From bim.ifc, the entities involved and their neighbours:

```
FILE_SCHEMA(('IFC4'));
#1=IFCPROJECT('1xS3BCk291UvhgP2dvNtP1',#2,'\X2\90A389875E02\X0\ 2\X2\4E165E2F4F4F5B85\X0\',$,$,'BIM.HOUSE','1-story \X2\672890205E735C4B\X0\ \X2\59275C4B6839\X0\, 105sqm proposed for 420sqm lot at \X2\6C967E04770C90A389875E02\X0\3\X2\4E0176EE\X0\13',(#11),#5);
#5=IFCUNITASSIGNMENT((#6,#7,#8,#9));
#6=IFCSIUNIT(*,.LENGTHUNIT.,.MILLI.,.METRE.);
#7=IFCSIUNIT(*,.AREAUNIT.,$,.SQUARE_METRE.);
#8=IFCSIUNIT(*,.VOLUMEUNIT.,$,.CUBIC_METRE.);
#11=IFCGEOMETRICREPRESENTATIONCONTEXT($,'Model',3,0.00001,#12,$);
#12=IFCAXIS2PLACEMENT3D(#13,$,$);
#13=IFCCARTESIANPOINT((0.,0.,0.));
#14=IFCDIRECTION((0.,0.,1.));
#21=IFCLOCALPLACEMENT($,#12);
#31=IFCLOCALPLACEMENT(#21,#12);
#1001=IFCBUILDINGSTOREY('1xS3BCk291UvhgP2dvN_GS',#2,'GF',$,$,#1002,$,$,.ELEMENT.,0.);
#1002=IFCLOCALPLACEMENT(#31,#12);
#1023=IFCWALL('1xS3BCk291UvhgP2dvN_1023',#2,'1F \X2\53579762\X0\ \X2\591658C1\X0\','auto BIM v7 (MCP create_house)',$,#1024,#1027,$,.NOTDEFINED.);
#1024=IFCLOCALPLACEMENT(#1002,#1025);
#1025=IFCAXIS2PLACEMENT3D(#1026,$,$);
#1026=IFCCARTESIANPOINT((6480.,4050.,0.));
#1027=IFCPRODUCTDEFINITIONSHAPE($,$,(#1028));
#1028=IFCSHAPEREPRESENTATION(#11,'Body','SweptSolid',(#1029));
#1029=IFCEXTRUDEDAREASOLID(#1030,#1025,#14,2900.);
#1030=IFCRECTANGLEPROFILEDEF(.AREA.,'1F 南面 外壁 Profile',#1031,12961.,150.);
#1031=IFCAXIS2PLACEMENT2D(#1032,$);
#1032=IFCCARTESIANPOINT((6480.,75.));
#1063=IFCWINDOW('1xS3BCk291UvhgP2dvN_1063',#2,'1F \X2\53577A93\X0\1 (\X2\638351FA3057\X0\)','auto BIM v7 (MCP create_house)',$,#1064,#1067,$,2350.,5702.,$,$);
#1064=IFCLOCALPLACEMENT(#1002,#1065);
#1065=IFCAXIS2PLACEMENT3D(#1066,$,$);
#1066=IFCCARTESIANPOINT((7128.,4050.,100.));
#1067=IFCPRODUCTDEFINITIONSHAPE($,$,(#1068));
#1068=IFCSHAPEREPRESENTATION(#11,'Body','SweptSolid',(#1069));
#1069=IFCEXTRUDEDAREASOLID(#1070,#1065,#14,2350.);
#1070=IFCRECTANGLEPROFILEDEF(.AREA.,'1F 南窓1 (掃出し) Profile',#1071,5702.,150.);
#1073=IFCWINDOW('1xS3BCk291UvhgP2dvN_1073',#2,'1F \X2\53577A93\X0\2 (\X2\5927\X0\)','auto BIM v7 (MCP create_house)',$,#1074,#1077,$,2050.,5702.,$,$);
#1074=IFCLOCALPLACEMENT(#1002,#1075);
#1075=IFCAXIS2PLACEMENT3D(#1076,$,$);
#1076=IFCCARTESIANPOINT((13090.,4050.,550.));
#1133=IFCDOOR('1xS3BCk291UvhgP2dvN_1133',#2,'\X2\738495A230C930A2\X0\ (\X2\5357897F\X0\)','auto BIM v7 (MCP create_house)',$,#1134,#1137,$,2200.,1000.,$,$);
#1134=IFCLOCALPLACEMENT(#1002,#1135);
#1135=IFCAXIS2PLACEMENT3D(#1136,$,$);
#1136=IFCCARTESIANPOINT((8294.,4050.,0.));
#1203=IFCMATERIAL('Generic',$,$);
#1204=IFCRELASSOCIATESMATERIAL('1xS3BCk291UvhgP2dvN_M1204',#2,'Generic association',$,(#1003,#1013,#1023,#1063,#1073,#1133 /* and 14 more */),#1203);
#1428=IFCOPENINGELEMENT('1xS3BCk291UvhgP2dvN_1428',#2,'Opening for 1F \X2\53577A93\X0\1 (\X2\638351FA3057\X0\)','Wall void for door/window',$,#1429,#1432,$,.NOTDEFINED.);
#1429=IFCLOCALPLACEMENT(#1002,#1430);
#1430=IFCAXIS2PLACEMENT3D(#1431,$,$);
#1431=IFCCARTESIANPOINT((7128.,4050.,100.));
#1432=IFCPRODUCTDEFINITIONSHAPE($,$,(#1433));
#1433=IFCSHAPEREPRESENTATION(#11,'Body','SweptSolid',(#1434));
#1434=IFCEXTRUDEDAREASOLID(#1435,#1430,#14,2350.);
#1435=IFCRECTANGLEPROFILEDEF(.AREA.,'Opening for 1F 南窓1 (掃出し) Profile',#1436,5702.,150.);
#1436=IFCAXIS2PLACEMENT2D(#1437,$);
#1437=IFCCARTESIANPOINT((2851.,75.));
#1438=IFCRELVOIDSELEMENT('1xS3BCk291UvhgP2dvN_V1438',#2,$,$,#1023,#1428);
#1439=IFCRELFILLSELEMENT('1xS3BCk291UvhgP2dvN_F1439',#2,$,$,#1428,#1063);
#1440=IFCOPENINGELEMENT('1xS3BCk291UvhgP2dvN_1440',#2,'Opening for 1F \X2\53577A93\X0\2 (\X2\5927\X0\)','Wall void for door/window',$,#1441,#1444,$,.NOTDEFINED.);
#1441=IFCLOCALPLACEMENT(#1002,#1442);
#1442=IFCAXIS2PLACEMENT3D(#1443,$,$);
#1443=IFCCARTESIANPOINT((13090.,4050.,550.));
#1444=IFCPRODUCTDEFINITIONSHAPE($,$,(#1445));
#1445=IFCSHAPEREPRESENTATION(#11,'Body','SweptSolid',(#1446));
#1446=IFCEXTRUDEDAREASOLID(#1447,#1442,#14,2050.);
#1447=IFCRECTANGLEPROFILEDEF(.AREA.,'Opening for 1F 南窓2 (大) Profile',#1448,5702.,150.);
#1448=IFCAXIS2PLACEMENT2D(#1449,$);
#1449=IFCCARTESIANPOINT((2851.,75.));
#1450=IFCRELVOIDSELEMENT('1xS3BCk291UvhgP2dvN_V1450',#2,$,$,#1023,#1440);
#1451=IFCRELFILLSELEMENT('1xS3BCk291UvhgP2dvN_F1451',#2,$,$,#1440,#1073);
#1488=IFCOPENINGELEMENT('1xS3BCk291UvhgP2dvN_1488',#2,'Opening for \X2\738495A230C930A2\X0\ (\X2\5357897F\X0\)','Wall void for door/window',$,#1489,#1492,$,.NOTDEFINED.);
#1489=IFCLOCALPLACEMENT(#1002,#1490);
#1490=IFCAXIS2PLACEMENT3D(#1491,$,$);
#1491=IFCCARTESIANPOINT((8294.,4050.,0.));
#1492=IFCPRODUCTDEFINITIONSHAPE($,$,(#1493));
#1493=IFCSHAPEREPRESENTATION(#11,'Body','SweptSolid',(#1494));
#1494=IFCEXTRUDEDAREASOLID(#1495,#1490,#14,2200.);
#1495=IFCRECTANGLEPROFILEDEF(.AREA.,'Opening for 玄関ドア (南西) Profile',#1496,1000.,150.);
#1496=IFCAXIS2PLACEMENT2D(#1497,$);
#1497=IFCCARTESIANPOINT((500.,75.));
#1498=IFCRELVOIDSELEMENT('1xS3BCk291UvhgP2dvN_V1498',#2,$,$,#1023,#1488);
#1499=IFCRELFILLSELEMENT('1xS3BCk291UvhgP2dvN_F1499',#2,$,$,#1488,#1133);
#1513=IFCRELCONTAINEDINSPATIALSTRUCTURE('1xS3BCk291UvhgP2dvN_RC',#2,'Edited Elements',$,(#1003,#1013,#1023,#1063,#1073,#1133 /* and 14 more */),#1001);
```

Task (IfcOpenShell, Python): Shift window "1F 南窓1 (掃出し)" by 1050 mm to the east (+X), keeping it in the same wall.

```python
import ifcopenshell
import ifcopenshell.api.geometry
import ifcopenshell.util.placement

model = ifcopenshell.open("bim.ifc")

window = model.by_id(1063)
opening = window.FillsVoids[0].RelatingOpeningElement
wall = opening.VoidsElements[0].RelatingBuildingElement

wall_matrix = ifcopenshell.util.placement.get_local_placement(wall.ObjectPlacement)
shift = wall_matrix[:3, 0] * 1050.0
before = ifcopenshell.util.placement.get_local_placement(window.ObjectPlacement)[:3, 3].copy()

# The window is not placed relative to its opening, so move both.
for product in (opening, window):
    matrix = ifcopenshell.util.placement.get_local_placement(product.ObjectPlacement)
    matrix[:3, 3] += shift
    ifcopenshell.api.geometry.edit_object_placement(model, product=product, matrix=matrix, is_si=False)

after = ifcopenshell.util.placement.get_local_placement(window.ObjectPlacement)[:3, 3]
print("window moved by", (after - before).round(3) + 0.0)

model.write("bim_updated.ifc")
```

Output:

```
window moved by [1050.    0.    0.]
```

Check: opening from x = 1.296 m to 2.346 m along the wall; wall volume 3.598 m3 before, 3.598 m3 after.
